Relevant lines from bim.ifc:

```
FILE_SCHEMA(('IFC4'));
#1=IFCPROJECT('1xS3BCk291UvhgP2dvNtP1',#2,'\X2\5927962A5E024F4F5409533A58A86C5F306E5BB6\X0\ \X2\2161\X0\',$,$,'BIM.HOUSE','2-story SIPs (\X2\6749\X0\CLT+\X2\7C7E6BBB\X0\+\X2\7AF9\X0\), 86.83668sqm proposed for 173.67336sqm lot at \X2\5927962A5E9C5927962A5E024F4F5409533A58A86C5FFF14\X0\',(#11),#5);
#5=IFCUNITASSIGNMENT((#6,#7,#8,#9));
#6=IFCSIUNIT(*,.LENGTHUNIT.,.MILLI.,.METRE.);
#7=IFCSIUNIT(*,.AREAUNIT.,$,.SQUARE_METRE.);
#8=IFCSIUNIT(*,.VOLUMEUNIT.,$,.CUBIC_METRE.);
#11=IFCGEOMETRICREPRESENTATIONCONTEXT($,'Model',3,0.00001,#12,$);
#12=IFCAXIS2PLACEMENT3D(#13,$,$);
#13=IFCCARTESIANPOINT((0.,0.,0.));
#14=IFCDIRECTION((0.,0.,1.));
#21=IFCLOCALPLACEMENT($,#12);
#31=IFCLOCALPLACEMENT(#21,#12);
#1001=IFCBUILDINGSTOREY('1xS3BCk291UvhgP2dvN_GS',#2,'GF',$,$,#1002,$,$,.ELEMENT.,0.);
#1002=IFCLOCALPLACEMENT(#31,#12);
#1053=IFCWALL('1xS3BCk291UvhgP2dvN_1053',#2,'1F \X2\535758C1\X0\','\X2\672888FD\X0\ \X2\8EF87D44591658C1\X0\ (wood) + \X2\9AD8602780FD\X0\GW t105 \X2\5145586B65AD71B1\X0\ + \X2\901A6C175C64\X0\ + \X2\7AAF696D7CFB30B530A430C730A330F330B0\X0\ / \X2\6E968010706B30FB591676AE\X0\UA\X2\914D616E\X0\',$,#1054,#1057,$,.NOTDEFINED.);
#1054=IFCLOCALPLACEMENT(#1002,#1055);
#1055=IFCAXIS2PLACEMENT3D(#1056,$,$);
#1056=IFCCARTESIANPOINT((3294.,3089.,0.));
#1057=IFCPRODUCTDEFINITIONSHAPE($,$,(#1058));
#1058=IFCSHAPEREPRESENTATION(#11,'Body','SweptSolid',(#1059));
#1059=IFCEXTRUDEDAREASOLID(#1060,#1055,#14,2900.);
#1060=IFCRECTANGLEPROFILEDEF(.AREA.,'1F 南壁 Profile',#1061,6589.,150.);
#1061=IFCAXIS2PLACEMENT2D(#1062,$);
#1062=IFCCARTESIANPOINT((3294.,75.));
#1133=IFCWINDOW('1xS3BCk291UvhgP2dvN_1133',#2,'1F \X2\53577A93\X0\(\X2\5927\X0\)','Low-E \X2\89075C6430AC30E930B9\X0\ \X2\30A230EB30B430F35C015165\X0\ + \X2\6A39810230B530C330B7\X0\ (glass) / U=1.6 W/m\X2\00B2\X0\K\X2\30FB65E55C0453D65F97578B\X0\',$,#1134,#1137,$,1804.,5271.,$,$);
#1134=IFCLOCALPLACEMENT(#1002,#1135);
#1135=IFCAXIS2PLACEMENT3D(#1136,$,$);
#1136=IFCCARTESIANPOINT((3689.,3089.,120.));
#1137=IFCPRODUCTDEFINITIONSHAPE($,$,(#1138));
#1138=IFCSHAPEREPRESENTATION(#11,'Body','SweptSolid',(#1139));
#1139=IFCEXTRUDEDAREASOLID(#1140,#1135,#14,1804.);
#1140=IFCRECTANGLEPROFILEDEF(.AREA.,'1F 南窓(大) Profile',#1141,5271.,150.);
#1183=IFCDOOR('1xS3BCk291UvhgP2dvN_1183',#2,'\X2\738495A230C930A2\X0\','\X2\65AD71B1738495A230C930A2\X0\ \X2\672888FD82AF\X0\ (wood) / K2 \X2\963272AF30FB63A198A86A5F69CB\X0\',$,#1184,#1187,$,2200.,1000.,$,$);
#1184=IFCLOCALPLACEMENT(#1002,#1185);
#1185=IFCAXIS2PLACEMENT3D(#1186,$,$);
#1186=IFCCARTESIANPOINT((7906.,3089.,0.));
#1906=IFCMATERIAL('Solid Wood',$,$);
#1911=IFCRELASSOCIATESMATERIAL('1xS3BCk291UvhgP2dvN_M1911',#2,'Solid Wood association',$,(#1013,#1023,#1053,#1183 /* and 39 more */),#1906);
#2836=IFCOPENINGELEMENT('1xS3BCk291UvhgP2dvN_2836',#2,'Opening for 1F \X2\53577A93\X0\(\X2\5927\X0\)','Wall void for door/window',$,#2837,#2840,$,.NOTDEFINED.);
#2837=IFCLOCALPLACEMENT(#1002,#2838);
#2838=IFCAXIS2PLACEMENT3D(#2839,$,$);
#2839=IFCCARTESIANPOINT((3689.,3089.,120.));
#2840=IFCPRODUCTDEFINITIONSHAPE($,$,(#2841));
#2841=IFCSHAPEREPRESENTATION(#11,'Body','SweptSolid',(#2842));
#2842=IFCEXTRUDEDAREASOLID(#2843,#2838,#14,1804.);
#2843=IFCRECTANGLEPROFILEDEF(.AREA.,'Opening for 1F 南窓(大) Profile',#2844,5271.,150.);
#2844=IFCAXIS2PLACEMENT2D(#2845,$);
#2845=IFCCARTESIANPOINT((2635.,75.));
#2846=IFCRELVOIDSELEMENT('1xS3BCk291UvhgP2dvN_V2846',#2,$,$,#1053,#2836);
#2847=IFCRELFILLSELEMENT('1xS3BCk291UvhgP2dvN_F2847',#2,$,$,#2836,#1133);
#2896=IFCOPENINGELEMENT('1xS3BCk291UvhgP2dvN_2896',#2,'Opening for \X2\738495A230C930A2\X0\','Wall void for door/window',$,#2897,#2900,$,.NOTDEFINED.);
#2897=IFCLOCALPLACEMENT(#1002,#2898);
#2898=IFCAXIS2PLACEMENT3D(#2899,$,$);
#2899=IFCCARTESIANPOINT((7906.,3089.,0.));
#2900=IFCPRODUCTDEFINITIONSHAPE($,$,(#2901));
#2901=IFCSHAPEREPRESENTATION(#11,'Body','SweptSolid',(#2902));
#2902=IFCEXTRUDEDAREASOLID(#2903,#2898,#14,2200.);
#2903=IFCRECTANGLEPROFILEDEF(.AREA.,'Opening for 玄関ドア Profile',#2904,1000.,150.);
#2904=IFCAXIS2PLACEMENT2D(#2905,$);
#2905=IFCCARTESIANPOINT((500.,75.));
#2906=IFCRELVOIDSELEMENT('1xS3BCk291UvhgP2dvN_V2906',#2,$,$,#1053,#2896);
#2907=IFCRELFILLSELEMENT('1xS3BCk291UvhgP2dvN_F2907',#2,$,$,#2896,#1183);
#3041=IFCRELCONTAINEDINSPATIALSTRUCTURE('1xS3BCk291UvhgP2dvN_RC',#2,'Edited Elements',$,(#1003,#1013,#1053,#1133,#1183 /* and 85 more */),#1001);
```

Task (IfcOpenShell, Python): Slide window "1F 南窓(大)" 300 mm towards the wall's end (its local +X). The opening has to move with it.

```python
import ifcopenshell
import ifcopenshell.api.geometry
import ifcopenshell.util.placement
import ifcopenshell.util.unit

model = ifcopenshell.open("bim.ifc")
unit_scale = ifcopenshell.util.unit.calculate_unit_scale(model)

window = model.by_guid("1xS3BCk291UvhgP2dvN_1133")
opening = window.FillsVoids[0].RelatingOpeningElement
wall = opening.VoidsElements[0].RelatingBuildingElement

wall_matrix = ifcopenshell.util.placement.get_local_placement(wall.ObjectPlacement)
shift = wall_matrix[:3, 0] * 0.3 / unit_scale
before = ifcopenshell.util.placement.get_local_placement(window.ObjectPlacement)[:3, 3].copy()

# The window is not placed relative to its opening, so move both.
for product in (opening, window):
    matrix = ifcopenshell.util.placement.get_local_placement(product.ObjectPlacement)
    matrix[:3, 3] += shift
    ifcopenshell.api.geometry.edit_object_placement(model, product=product, matrix=matrix, is_si=False)

after = ifcopenshell.util.placement.get_local_placement(window.ObjectPlacement)[:3, 3]
print("window moved by", (after - before).round(3) + 0.0)

model.write("bim_updated.ifc")
```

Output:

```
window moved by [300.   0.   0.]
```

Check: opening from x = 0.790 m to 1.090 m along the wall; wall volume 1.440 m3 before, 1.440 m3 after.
